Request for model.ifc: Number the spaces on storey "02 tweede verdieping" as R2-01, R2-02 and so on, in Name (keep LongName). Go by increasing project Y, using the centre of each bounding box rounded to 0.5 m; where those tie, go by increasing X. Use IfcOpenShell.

First a look at what the model holds.

```python
import ifcopenshell
import ifcopenshell.util.element
import ifcopenshell.util.placement

model = ifcopenshell.open("model.ifc")
print(model.schema)
storey = next(s for s in model.by_type("IfcBuildingStorey") if s.Name == "02 tweede verdieping")
spaces = [e for e in ifcopenshell.util.element.get_decomposition(storey) if e.is_a("IfcSpace")]
for e in sorted(spaces, key=lambda e: e.id()):
    origin = ifcopenshell.util.placement.get_local_placement(e.ObjectPlacement)[:3, 3]
    print(e.id(), e.Name, e.LongName, origin.round(2) + 0.0, sep=" | ")
```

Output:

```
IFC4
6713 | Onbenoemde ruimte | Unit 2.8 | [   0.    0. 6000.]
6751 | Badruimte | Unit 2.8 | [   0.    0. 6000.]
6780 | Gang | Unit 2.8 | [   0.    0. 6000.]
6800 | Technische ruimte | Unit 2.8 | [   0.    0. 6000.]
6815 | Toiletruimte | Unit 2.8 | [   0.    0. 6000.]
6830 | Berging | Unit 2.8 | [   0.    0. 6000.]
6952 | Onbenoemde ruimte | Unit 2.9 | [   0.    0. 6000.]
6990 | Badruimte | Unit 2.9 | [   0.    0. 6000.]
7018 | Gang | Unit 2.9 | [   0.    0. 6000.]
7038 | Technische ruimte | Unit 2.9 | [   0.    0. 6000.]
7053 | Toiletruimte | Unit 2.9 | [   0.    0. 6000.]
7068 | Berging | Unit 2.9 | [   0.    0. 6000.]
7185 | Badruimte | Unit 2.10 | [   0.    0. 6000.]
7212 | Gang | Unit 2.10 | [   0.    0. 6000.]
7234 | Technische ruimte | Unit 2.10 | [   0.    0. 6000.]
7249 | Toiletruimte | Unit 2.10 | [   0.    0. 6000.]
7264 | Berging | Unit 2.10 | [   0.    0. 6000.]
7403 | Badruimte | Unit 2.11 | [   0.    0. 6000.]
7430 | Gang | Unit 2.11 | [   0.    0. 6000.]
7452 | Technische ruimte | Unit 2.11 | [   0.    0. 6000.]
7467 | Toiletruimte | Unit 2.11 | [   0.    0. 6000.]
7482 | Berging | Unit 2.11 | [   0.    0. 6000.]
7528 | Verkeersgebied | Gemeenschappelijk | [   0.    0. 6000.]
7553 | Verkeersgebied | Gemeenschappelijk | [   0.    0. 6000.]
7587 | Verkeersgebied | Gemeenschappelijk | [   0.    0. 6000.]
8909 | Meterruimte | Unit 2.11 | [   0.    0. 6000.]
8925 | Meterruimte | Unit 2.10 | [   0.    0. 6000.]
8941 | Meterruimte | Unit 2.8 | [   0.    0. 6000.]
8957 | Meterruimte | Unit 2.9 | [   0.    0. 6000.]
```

```python
import ifcopenshell
import ifcopenshell.geom
import ifcopenshell.util.element
import ifcopenshell.util.shape

model = ifcopenshell.open("model.ifc")
settings = ifcopenshell.geom.settings()
settings.set("use-world-coords", True)


def centre(element):
    shape = ifcopenshell.geom.create_shape(settings, element)
    return ifcopenshell.util.shape.get_bbox_centroid(shape.geometry)


storey = next(s for s in model.by_type("IfcBuildingStorey") if s.Name == "02 tweede verdieping")
spaces = [e for e in ifcopenshell.util.element.get_decomposition(storey) if e.is_a("IfcSpace")]

# Insertion points can sit at a corner or the storey origin, so sort by the geometry (in metres).
centres = {e: centre(e) for e in spaces}
spaces.sort(key=lambda e: (round(centres[e][1] / 0.5), centres[e][0]))

for i, e in enumerate(spaces, start=1):
    number = f"R2-{i:02d}"
    e.Name = number
    print(e.id(), number)

model.write("model_edited.ifc")
```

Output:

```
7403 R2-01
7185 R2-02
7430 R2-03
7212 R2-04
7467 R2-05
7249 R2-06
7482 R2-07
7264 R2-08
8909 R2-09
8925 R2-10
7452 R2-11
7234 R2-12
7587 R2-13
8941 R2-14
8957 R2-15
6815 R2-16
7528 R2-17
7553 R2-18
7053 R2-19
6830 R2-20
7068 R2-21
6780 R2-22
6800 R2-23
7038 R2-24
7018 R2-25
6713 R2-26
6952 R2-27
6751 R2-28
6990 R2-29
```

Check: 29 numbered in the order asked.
